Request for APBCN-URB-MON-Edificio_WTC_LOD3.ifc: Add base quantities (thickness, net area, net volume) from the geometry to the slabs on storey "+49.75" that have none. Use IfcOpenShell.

First a look at what the model holds.

```python
import ifcopenshell
import ifcopenshell.util.element
import ifcopenshell.util.unit

model = ifcopenshell.open("APBCN-URB-MON-Edificio_WTC_LOD3.ifc")
print(model.schema)
for unit_type in ("LENGTHUNIT", "AREAUNIT", "VOLUMEUNIT"):
    print(unit_type, ifcopenshell.util.unit.calculate_unit_scale(model, unit_type))
storey = next(s for s in model.by_type("IfcBuildingStorey") if s.Name == "+49.75")
slabs = [e for e in ifcopenshell.util.element.get_decomposition(storey) if e.is_a("IfcSlab")]
for e in sorted(slabs, key=lambda e: e.id()):
    print(e.id(), e.is_a(), e.Name, list(ifcopenshell.util.element.get_psets(e, qtos_only=True)), sep=" | ")
```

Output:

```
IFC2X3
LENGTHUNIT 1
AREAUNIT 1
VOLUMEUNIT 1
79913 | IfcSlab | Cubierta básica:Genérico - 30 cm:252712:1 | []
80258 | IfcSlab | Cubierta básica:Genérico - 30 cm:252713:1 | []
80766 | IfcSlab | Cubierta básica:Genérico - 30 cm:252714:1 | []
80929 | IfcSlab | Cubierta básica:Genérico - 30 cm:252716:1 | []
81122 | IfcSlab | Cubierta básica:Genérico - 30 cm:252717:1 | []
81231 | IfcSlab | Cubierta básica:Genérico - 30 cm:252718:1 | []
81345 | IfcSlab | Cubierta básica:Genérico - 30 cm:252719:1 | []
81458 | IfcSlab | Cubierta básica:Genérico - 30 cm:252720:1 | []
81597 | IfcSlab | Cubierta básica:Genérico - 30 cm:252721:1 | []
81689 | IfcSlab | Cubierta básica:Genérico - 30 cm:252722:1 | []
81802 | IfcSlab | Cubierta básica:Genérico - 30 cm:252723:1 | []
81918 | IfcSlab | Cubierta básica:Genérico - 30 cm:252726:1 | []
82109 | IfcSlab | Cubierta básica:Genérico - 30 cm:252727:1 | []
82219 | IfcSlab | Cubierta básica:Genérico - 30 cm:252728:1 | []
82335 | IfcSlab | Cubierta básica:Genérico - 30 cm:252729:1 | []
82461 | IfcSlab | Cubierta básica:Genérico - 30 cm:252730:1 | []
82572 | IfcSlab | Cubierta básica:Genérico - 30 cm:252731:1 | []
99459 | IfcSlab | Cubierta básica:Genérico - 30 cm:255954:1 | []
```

```python
import ifcopenshell
import ifcopenshell.api.pset
import ifcopenshell.geom
import ifcopenshell.util.element
import ifcopenshell.util.shape
import ifcopenshell.util.unit

model = ifcopenshell.open("APBCN-URB-MON-Edificio_WTC_LOD3.ifc")
unit_scale = ifcopenshell.util.unit.calculate_unit_scale(model)
area_scale = ifcopenshell.util.unit.calculate_unit_scale(model, "AREAUNIT")
volume_scale = ifcopenshell.util.unit.calculate_unit_scale(model, "VOLUMEUNIT")
settings = ifcopenshell.geom.settings()

storey = next(s for s in model.by_type("IfcBuildingStorey") if s.Name == "+49.75")
slabs = [e for e in ifcopenshell.util.element.get_decomposition(storey) if e.is_a("IfcSlab")]

for e in sorted(slabs, key=lambda e: e.id()):
    if ifcopenshell.util.element.get_psets(e, qtos_only=True, should_inherit=False):
        continue
    # Geometry comes back in metres, in the element's own axes.
    shape = ifcopenshell.geom.create_shape(settings, e)
    values = {
        "Width": ifcopenshell.util.shape.get_z(shape.geometry) / unit_scale,
        "NetArea": ifcopenshell.util.shape.get_footprint_area(shape.geometry) / area_scale,
        "NetVolume": ifcopenshell.util.shape.get_volume(shape.geometry) / volume_scale,
    }
    qto = ifcopenshell.api.pset.add_qto(model, product=e, name="BaseQuantities")
    ifcopenshell.api.pset.edit_qto(model, qto=qto, properties=values)
    print(e.id(), {k: round(v, 3) for k, v in values.items()})

model.write("APBCN-URB-MON-Edificio_WTC_LOD3-out.ifc")
```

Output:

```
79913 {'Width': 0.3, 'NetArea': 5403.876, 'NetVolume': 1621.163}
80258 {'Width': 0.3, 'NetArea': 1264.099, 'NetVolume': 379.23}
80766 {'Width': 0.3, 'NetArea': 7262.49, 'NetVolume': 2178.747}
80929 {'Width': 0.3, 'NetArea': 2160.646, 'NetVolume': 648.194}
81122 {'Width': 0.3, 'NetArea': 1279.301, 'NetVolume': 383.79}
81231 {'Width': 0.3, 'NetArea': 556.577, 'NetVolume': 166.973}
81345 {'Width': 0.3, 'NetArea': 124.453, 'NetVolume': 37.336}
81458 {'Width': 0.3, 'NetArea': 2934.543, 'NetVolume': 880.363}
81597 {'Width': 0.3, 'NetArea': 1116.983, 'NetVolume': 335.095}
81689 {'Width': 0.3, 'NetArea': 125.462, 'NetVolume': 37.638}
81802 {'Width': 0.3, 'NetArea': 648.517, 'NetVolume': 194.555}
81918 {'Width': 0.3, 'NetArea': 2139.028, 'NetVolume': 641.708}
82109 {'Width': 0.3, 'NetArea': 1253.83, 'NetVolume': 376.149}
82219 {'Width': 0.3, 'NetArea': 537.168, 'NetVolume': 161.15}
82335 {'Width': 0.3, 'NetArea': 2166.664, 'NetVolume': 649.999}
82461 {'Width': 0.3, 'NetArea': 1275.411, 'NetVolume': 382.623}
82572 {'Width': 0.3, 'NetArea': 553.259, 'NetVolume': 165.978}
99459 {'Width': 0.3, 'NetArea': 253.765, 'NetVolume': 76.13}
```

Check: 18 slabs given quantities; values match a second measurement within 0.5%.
